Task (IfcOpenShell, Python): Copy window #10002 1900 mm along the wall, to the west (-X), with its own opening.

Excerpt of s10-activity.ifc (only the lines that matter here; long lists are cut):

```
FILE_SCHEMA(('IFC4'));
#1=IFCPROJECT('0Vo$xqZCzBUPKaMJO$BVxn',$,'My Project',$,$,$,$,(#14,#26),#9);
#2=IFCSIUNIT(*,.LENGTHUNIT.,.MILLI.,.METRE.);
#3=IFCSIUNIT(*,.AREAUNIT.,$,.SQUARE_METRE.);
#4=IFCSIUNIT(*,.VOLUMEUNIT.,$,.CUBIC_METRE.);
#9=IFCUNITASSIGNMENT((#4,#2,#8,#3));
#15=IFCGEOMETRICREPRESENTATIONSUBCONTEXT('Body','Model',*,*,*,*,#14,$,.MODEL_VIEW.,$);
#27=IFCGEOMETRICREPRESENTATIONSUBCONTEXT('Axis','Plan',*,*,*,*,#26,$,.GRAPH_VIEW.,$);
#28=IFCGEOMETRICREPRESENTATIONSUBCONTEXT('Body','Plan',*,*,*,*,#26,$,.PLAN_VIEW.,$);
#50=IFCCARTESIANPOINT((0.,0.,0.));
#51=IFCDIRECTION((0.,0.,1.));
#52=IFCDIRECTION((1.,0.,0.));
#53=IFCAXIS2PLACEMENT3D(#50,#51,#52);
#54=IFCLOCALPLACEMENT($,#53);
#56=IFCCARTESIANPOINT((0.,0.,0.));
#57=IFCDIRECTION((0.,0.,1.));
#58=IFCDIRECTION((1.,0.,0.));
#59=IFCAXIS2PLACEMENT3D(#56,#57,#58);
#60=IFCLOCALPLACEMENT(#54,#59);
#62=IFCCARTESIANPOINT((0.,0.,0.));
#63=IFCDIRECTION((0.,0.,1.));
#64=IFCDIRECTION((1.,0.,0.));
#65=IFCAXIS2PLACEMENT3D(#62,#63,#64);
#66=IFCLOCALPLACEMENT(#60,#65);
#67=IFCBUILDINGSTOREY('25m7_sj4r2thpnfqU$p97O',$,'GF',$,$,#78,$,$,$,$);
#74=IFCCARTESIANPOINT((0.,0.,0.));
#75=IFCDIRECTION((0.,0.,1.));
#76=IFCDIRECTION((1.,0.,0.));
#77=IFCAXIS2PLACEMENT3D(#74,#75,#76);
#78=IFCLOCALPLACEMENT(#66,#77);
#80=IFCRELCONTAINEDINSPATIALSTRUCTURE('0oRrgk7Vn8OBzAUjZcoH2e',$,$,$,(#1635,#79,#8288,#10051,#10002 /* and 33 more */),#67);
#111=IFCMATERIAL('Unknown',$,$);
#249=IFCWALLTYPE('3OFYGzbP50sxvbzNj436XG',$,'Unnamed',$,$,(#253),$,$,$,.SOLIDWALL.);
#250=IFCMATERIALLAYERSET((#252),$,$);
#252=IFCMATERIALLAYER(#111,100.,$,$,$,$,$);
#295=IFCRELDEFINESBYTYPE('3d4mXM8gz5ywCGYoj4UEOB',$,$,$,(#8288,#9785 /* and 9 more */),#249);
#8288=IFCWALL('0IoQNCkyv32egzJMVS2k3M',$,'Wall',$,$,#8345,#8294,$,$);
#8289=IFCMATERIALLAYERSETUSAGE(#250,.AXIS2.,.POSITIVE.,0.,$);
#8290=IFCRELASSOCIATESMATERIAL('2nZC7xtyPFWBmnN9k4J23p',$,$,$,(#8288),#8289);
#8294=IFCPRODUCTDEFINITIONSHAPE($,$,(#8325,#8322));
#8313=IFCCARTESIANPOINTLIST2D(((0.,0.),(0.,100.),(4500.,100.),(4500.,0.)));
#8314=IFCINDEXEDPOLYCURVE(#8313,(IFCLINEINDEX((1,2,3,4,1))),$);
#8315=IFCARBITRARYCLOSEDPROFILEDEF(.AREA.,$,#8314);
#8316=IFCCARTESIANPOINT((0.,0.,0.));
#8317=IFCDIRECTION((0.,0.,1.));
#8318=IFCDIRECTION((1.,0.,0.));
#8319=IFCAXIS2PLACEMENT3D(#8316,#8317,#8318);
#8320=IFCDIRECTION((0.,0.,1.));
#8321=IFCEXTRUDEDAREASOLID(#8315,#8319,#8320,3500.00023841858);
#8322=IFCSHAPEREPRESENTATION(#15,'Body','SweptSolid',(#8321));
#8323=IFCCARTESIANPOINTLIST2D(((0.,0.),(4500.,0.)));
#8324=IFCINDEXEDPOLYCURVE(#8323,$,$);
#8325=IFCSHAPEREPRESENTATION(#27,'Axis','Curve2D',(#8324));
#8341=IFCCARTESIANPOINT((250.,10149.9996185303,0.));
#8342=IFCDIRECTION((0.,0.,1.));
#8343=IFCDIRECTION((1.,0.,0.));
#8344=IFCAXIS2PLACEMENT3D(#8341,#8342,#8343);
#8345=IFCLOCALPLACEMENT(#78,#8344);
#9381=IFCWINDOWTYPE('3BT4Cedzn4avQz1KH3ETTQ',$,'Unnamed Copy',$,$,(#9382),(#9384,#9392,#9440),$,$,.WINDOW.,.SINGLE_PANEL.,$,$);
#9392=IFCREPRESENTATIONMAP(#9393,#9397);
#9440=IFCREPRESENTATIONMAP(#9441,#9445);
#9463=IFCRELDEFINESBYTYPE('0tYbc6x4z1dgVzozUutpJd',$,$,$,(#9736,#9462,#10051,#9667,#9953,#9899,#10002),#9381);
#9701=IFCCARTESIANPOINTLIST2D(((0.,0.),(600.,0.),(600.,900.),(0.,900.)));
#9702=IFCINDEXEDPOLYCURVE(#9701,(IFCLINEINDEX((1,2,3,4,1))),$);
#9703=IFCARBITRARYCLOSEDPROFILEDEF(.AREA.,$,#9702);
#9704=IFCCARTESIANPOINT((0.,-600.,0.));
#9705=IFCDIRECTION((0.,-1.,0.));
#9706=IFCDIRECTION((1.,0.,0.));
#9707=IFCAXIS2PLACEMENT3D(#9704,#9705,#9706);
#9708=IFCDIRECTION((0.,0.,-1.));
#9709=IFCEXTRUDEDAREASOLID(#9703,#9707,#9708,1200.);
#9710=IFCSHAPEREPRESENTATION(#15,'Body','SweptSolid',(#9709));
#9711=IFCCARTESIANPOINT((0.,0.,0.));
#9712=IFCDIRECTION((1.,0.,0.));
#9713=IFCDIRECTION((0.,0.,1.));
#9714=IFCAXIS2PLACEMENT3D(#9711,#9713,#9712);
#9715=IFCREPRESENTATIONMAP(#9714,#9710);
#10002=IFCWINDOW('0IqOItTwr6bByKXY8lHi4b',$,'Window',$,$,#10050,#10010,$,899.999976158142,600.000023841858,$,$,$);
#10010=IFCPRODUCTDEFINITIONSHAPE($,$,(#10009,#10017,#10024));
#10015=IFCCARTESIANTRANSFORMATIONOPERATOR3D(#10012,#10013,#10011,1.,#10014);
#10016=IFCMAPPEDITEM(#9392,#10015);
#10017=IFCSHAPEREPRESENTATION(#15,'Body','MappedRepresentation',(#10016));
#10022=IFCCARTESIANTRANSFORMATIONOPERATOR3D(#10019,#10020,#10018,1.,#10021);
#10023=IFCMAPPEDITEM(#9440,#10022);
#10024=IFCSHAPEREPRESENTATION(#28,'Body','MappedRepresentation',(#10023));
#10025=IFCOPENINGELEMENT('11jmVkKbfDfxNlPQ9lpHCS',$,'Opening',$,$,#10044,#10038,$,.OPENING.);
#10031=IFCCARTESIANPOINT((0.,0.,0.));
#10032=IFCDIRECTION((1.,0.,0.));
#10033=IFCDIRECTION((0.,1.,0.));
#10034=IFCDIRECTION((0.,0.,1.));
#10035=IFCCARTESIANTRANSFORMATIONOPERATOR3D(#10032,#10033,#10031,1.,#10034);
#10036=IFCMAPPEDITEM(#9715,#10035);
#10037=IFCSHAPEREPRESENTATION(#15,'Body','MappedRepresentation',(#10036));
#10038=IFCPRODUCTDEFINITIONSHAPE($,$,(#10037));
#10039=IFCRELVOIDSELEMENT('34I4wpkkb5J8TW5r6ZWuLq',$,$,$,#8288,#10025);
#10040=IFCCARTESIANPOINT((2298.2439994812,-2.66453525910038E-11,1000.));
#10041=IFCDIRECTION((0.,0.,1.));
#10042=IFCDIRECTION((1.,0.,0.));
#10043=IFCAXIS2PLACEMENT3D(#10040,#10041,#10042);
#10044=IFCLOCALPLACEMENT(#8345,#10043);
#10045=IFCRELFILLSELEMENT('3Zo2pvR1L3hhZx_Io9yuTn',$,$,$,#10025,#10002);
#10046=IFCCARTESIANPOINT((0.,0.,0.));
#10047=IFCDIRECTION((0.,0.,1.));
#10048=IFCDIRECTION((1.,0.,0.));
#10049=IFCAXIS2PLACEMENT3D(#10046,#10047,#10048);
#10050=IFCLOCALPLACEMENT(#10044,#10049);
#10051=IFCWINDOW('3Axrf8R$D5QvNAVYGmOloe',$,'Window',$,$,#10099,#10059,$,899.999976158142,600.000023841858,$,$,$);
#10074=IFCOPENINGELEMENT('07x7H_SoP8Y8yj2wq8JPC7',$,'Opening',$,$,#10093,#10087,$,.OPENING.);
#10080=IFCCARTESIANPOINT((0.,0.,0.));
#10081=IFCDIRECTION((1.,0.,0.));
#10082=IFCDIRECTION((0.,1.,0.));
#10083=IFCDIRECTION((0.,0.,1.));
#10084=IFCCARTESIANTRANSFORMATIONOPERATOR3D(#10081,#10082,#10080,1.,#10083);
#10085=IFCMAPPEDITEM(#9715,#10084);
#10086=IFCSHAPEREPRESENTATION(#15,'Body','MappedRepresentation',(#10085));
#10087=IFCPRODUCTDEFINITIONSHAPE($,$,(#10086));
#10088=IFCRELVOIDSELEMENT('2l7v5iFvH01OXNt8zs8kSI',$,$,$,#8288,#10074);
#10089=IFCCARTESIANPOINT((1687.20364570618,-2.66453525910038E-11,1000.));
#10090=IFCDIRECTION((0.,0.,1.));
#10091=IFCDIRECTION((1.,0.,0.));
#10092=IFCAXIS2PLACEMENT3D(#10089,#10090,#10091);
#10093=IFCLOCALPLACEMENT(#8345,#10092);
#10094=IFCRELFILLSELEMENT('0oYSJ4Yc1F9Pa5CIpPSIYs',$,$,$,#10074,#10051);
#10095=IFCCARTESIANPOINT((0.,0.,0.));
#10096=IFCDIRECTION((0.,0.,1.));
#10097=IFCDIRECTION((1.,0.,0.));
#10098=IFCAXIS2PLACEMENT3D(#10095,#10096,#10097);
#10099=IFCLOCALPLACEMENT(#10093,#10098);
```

```python
import ifcopenshell
import ifcopenshell.api.feature
import ifcopenshell.api.geometry
import ifcopenshell.api.root
import ifcopenshell.geom
import ifcopenshell.util.element
import ifcopenshell.util.placement
import ifcopenshell.util.shape
import ifcopenshell.util.unit

model = ifcopenshell.open("s10-activity.ifc")
unit_scale = ifcopenshell.util.unit.calculate_unit_scale(model)
settings = ifcopenshell.geom.settings()


def volume(element):
    """Net volume in cubic metres, openings subtracted."""
    shape = ifcopenshell.geom.create_shape(settings, element)
    return ifcopenshell.util.shape.get_volume(shape.geometry)


window = model.by_guid("0IqOItTwr6bByKXY8lHi4b")
opening = window.FillsVoids[0].RelatingOpeningElement
wall = opening.VoidsElements[0].RelatingBuildingElement
before = volume(wall)
shift = ifcopenshell.util.placement.get_local_placement(wall.ObjectPlacement)[:3, 0] * -1.9 / unit_scale

# copy_class copies the void relationship, type, container and properties, but no geometry.
new_opening = ifcopenshell.api.root.copy_class(model, product=opening)
new_opening.Representation = ifcopenshell.util.element.copy_deep(
    model, opening.Representation, exclude=["IfcGeometricRepresentationContext", "IfcRepresentationMap"]
)
new_window = ifcopenshell.api.root.copy_class(model, product=window)
new_window.Representation = ifcopenshell.util.element.copy_deep(
    model, window.Representation, exclude=["IfcGeometricRepresentationContext", "IfcRepresentationMap"]
)
ifcopenshell.api.feature.add_filling(model, opening=new_opening, element=new_window)

for old, new in ((opening, new_opening), (window, new_window)):
    matrix = ifcopenshell.util.placement.get_local_placement(old.ObjectPlacement)
    matrix[:3, 3] += shift
    ifcopenshell.api.geometry.edit_object_placement(model, product=new, matrix=matrix, is_si=False)

after = volume(wall)

print(f"wall volume {before:.3f} -> {after:.3f} m3")

model.write("s10-activity_updated.ifc")
```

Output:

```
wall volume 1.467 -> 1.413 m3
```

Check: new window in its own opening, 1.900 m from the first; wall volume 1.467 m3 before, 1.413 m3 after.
